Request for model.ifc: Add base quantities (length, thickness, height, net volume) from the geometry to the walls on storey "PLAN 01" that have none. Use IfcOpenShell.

First a look at what the model holds.

```python
import ifcopenshell
import ifcopenshell.util.element
import ifcopenshell.util.unit

model = ifcopenshell.open("model.ifc")
print(model.schema)
for unit_type in ("LENGTHUNIT", "AREAUNIT", "VOLUMEUNIT"):
    print(unit_type, ifcopenshell.util.unit.calculate_unit_scale(model, unit_type))
storey = next(s for s in model.by_type("IfcBuildingStorey") if s.Name == "PLAN 01")
walls = [e for e in ifcopenshell.util.element.get_decomposition(storey) if e.is_a("IfcWall")]
for e in sorted(walls, key=lambda e: e.id()):
    print(e.id(), e.is_a(), e.Name, list(ifcopenshell.util.element.get_psets(e, qtos_only=True)), sep=" | ")
```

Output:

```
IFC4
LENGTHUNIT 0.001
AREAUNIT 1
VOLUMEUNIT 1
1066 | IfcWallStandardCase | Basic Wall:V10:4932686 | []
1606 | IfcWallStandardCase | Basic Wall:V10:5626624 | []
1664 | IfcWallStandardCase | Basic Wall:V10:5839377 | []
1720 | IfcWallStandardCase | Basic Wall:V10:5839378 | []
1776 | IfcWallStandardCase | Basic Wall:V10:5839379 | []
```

```python
import ifcopenshell
import ifcopenshell.api.pset
import ifcopenshell.geom
import ifcopenshell.util.element
import ifcopenshell.util.shape
import ifcopenshell.util.unit

model = ifcopenshell.open("model.ifc")
unit_scale = ifcopenshell.util.unit.calculate_unit_scale(model)
volume_scale = ifcopenshell.util.unit.calculate_unit_scale(model, "VOLUMEUNIT")
settings = ifcopenshell.geom.settings()

storey = next(s for s in model.by_type("IfcBuildingStorey") if s.Name == "PLAN 01")
walls = [e for e in ifcopenshell.util.element.get_decomposition(storey) if e.is_a("IfcWall")]

for e in sorted(walls, key=lambda e: e.id()):
    if ifcopenshell.util.element.get_psets(e, qtos_only=True, should_inherit=False):
        continue
    # Geometry comes back in metres, in the element's own axes.
    shape = ifcopenshell.geom.create_shape(settings, e)
    values = {
        "Length": ifcopenshell.util.shape.get_x(shape.geometry) / unit_scale,
        "Width": ifcopenshell.util.shape.get_y(shape.geometry) / unit_scale,
        "Height": ifcopenshell.util.shape.get_z(shape.geometry) / unit_scale,
        "NetVolume": ifcopenshell.util.shape.get_volume(shape.geometry) / volume_scale,
    }
    qto = ifcopenshell.api.pset.add_qto(model, product=e, name="Qto_WallBaseQuantities")
    ifcopenshell.api.pset.edit_qto(model, qto=qto, properties=values)
    print(e.id(), {k: round(v, 3) for k, v in values.items()})

model.write("model_updated.ifc")
```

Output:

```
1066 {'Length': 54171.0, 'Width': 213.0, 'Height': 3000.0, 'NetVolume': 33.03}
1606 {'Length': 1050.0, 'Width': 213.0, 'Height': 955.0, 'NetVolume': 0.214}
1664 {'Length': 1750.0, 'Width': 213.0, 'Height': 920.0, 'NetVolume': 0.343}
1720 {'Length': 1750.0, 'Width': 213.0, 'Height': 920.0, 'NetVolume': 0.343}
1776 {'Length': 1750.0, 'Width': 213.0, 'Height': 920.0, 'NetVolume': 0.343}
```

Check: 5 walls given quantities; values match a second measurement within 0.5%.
